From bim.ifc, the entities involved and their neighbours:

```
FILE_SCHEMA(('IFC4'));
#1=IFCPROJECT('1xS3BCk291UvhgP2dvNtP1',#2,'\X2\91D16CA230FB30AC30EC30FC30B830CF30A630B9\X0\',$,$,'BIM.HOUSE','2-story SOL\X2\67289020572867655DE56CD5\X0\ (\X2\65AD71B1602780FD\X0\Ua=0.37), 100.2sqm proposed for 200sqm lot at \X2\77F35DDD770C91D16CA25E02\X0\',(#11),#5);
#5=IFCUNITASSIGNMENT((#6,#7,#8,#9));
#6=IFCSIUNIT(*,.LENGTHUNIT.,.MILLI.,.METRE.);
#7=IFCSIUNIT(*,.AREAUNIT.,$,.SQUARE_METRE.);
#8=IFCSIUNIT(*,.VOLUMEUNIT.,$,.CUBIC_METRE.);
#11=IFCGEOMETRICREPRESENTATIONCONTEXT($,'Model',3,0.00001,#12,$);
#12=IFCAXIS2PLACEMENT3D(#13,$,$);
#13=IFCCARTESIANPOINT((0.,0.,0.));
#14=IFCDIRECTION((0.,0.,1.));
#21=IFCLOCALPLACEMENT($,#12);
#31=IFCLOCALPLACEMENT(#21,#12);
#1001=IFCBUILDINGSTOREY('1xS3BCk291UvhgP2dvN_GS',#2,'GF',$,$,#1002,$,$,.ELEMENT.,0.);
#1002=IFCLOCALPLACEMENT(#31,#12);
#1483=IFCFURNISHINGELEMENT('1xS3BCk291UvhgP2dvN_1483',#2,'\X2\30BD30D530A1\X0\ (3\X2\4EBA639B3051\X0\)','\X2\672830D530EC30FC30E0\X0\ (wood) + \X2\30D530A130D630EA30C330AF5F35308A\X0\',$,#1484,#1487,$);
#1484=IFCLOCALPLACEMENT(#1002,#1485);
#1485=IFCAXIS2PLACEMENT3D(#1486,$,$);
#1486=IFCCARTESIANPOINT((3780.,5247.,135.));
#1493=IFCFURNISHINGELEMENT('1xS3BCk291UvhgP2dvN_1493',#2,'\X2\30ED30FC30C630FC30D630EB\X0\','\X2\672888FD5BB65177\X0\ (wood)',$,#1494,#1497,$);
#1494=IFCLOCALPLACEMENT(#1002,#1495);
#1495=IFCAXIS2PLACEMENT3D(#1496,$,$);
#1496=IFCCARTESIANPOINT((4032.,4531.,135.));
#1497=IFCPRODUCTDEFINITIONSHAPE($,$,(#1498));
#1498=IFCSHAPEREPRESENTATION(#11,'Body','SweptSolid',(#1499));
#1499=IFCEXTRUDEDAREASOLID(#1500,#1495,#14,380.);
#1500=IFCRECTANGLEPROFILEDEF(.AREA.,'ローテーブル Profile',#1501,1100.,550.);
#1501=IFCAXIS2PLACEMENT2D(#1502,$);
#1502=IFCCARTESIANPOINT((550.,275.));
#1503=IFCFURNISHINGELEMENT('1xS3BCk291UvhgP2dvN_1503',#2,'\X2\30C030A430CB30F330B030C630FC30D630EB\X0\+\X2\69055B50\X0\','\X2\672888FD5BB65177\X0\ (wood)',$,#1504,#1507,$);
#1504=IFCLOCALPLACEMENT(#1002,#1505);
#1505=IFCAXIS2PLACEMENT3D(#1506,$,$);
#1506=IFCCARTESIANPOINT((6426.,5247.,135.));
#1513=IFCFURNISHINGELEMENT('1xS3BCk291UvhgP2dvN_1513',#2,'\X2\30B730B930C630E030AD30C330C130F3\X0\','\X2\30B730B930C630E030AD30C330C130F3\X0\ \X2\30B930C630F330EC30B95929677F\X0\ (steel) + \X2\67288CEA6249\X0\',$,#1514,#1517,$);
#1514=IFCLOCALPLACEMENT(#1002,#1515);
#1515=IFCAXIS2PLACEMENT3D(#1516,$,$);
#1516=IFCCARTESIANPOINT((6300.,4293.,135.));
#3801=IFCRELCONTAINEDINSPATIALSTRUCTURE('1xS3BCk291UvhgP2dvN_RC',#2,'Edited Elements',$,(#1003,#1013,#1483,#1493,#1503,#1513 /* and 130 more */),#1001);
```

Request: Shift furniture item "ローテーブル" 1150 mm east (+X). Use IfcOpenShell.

```python
import ifcopenshell
import ifcopenshell.api.geometry
import ifcopenshell.util.placement
import ifcopenshell.util.unit

model = ifcopenshell.open("bim.ifc")
unit_scale = ifcopenshell.util.unit.calculate_unit_scale(model)

item = model.by_guid("1xS3BCk291UvhgP2dvN_1493")
matrix = ifcopenshell.util.placement.get_local_placement(item.ObjectPlacement)
matrix[0, 3] += 1.15 / unit_scale
ifcopenshell.api.geometry.edit_object_placement(model, product=item, matrix=matrix, is_si=False)

print(ifcopenshell.util.placement.get_local_placement(item.ObjectPlacement).round(3) + 0.0)

model.write("bim_v2.ifc")
```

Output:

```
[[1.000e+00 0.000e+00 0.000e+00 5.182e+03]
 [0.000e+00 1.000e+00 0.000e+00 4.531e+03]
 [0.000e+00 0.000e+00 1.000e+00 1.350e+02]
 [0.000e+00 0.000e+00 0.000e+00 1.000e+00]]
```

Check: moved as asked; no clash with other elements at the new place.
